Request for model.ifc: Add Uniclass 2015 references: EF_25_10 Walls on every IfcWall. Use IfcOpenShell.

First a look at what the model holds.

```python
import ifcopenshell

model = ifcopenshell.open("model.ifc")
print(model.schema)
print("classifications:", [c.Name for c in model.by_type("IfcClassification")])
for ifc_class in ("IfcDoor", "IfcRoof", "IfcStair", "IfcWall", "IfcWindow"):
    print(ifc_class, len(model.by_type(ifc_class)))
```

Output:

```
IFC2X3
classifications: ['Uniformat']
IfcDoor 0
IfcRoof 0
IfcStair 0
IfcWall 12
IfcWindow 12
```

```python
import ifcopenshell
import ifcopenshell.api.classification

model = ifcopenshell.open("model.ifc")

# IFC2X3 requires Source and Edition and has no link from the project to the system.
system = model.create_entity("IfcClassification", Source="NBS", Edition="2015", Name="Uniclass 2015")

codes = {
    "IfcWall": ("EF_25_10", "Walls"),
}
for ifc_class, (code, name) in codes.items():
    products = model.by_type(ifc_class)
    ifcopenshell.api.classification.add_reference(
        model, products=products, classification=system, identification=code, name=name
    )
    print(code, len(products))

model.write("model_edited.ifc")
```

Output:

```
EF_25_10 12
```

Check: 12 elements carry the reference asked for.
